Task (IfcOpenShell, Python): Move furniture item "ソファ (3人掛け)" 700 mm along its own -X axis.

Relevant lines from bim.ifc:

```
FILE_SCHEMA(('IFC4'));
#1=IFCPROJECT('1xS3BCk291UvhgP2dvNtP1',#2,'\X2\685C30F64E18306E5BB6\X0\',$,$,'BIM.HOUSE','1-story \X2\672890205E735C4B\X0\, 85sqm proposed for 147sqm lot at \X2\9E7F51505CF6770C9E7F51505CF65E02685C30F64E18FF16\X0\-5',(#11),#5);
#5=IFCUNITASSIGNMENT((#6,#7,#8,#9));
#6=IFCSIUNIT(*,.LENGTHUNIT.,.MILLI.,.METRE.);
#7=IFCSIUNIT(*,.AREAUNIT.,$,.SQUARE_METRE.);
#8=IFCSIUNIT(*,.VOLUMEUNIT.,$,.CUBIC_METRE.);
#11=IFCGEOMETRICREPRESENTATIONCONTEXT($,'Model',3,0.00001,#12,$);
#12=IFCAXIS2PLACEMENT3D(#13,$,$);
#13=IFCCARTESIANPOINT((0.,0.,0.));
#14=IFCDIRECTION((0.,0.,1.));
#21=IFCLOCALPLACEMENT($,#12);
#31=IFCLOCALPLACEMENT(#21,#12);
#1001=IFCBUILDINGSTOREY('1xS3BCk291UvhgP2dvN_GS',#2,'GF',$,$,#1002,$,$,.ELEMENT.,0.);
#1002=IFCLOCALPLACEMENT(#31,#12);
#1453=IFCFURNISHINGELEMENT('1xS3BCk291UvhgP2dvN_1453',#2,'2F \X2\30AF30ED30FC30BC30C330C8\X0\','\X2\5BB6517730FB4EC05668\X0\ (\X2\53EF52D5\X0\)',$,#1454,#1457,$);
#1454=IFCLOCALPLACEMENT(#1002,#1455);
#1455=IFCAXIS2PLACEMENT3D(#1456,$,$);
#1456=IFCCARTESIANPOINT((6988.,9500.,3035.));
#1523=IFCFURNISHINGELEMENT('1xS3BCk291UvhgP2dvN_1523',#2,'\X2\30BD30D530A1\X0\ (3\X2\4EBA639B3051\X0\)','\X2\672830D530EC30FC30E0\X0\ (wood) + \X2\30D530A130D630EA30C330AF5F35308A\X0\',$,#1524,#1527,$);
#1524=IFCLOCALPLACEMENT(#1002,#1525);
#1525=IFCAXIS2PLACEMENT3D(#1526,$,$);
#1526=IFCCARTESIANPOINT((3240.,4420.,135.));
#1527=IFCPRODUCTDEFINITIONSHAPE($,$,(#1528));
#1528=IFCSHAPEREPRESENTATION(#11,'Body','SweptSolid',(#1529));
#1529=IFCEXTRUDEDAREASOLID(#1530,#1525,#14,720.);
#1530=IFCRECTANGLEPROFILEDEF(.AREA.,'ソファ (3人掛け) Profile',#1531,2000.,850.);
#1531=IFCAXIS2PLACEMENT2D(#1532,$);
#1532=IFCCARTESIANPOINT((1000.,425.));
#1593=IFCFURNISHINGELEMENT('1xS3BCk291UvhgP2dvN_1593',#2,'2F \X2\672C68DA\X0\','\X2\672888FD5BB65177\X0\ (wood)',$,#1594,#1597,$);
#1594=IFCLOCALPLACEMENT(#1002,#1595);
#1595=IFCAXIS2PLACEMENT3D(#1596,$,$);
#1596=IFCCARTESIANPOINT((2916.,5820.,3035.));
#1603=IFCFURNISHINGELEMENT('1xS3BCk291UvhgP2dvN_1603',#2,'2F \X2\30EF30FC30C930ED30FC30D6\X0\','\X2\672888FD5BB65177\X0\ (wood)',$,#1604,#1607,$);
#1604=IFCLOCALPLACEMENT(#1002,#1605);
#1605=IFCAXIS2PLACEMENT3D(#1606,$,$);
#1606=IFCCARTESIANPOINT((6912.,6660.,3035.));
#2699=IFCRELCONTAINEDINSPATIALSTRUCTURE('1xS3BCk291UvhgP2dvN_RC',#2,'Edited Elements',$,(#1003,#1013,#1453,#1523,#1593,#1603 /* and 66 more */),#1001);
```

```python
import ifcopenshell
import ifcopenshell.api.geometry
import ifcopenshell.util.placement

model = ifcopenshell.open("bim.ifc")

item = model.by_guid("1xS3BCk291UvhgP2dvN_1523")
matrix = ifcopenshell.util.placement.get_local_placement(item.ObjectPlacement)
matrix[:3, 3] -= matrix[:3, 0] * 700.0
ifcopenshell.api.geometry.edit_object_placement(model, product=item, matrix=matrix, is_si=False)

print(ifcopenshell.util.placement.get_local_placement(item.ObjectPlacement).round(3) + 0.0)

model.write("bim-out.ifc")
```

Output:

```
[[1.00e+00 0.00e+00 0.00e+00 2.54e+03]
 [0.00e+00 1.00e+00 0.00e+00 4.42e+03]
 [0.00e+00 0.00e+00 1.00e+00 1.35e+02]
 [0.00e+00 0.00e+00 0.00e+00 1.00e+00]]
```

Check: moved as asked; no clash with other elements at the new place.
